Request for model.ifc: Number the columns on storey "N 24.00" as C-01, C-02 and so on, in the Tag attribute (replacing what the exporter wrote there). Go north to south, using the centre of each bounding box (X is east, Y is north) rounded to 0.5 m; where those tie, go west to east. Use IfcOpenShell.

First a look at what the model holds.

```python
import ifcopenshell
import ifcopenshell.util.element
import ifcopenshell.util.placement

model = ifcopenshell.open("model.ifc")
print(model.schema)
storey = next(s for s in model.by_type("IfcBuildingStorey") if s.Name == "N 24.00")
columns = [e for e in ifcopenshell.util.element.get_decomposition(storey) if e.is_a("IfcColumn")]
for e in sorted(columns, key=lambda e: e.id()):
    origin = ifcopenshell.util.placement.get_local_placement(e.ObjectPlacement)[:3, 3]
    print(e.id(), e.Tag, e.Name, origin.round(2) + 0.0, sep=" | ")
```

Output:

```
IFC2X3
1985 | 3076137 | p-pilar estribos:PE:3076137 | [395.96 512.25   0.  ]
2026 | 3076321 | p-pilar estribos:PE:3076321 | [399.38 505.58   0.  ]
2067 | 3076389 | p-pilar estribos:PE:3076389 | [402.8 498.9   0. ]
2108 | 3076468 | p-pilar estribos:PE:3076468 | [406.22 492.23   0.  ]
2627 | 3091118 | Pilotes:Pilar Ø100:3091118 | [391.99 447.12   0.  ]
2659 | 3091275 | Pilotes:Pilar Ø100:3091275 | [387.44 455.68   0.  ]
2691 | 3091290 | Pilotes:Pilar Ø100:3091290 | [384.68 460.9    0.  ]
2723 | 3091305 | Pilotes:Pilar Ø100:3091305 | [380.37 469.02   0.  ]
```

```python
import ifcopenshell
import ifcopenshell.geom
import ifcopenshell.util.element
import ifcopenshell.util.shape

model = ifcopenshell.open("model.ifc")
settings = ifcopenshell.geom.settings()
settings.set("use-world-coords", True)


def centre(element):
    shape = ifcopenshell.geom.create_shape(settings, element)
    return ifcopenshell.util.shape.get_bbox_centroid(shape.geometry)


storey = next(s for s in model.by_type("IfcBuildingStorey") if s.Name == "N 24.00")
columns = [e for e in ifcopenshell.util.element.get_decomposition(storey) if e.is_a("IfcColumn")]

# Insertion points can sit at a corner or the storey origin, so sort by the geometry (in metres).
centres = {e: centre(e) for e in columns}
columns.sort(key=lambda e: (-round(centres[e][1] / 0.5), centres[e][0]))

for i, e in enumerate(columns, start=1):
    number = f"C-{i:02d}"
    e.Tag = number
    print(e.id(), number)

model.write("model_v2.ifc")
```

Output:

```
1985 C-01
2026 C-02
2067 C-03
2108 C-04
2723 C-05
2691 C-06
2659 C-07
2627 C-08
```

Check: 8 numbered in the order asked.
